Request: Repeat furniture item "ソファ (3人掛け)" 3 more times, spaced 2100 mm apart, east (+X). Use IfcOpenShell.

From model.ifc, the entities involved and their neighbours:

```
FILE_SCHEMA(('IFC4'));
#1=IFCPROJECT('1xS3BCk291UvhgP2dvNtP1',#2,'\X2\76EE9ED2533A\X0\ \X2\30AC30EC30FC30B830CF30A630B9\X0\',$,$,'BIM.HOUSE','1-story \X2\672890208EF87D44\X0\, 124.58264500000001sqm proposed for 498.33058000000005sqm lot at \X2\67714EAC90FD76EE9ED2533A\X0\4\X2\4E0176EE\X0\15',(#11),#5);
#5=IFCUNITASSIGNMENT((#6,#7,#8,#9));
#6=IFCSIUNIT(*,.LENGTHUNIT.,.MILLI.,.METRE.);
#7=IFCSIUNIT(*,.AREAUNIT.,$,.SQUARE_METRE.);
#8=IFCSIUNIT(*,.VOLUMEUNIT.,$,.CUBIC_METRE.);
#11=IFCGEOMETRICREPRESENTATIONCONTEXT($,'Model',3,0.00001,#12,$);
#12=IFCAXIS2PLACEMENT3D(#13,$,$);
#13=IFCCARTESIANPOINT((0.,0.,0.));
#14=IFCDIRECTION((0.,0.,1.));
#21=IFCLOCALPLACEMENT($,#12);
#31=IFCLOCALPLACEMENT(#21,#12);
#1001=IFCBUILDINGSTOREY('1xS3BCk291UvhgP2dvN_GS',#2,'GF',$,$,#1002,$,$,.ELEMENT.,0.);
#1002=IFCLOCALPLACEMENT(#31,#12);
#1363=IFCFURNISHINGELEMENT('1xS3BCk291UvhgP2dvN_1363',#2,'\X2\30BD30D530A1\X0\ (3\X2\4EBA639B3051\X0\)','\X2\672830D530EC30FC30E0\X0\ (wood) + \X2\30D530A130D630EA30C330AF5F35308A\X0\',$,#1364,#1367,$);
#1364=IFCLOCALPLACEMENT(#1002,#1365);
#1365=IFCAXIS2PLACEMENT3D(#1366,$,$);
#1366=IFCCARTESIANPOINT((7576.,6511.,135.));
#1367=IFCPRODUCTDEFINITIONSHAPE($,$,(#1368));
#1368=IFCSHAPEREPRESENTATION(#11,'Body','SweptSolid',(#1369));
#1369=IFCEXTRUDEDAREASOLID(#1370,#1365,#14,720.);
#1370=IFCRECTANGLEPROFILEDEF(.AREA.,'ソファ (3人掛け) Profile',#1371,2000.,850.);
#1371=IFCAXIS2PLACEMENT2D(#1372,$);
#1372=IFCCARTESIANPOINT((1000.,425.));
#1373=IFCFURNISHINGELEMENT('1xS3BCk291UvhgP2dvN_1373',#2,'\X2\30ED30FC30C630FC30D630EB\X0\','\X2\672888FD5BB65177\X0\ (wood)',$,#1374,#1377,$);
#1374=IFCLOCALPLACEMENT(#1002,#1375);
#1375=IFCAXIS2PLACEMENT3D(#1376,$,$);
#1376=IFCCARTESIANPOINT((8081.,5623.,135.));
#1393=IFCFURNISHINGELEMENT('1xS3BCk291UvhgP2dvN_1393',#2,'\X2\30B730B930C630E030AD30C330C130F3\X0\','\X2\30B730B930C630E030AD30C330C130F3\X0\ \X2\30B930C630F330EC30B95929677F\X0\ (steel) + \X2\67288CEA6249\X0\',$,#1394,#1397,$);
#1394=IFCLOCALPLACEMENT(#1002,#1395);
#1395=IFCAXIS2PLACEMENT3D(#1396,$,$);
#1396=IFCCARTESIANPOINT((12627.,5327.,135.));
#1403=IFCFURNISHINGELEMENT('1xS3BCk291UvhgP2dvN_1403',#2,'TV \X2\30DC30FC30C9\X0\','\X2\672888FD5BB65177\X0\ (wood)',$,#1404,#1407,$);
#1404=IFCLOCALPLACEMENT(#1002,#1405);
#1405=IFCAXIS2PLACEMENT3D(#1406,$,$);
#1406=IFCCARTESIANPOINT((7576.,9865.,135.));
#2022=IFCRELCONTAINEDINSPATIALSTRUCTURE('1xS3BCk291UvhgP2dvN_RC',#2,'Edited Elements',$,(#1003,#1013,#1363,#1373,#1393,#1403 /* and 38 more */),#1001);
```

```python
import numpy as np
import ifcopenshell
import ifcopenshell.api.geometry
import ifcopenshell.api.root
import ifcopenshell.util.element
import ifcopenshell.util.placement
import ifcopenshell.util.unit

model = ifcopenshell.open("model.ifc")
unit_scale = ifcopenshell.util.unit.calculate_unit_scale(model)


def reuse_history(source, copy):
    """copy_class also copies each property set's owner history, people and application; keep the originals."""
    for rel in copy.IsDefinedBy:
        if rel.is_a("IfcRelDefinesByProperties") and (history := rel.RelatingPropertyDefinition.OwnerHistory):
            rel.RelatingPropertyDefinition.OwnerHistory = source.OwnerHistory
            ifcopenshell.util.element.remove_deep2(model, history)


source = model.by_guid("1xS3BCk291UvhgP2dvN_1363")
base = ifcopenshell.util.placement.get_local_placement(source.ObjectPlacement)
step = np.array([1.0, 0.0, 0.0]) * 2.1 / unit_scale

for i in range(1, 4):
    copy = ifcopenshell.api.root.copy_class(model, product=source)
    copy.Representation = ifcopenshell.util.element.copy_deep(
        model, source.Representation, exclude=["IfcGeometricRepresentationContext", "IfcRepresentationMap"]
    )
    reuse_history(source, copy)
    matrix = base.copy()
    matrix[:3, 3] += i * step
    print("added at", matrix[:3, 3].round(3) + 0.0)
    ifcopenshell.api.geometry.edit_object_placement(model, product=copy, matrix=matrix, is_si=False)

model.write("model_edited.ifc")
```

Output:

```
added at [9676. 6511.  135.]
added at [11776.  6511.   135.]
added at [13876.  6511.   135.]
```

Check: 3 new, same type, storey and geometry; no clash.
